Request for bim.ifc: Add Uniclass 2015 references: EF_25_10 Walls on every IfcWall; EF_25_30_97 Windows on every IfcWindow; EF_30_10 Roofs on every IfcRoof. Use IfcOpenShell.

First a look at what the model holds.

```python
import ifcopenshell

model = ifcopenshell.open("bim.ifc")
print(model.schema)
print("classifications:", [c.Name for c in model.by_type("IfcClassification")])
for ifc_class in ("IfcDoor", "IfcRoof", "IfcStair", "IfcWall", "IfcWindow"):
    print(ifc_class, len(model.by_type(ifc_class)))
```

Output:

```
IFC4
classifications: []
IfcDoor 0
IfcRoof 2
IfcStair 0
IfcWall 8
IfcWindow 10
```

```python
import ifcopenshell
import ifcopenshell.api.classification

model = ifcopenshell.open("bim.ifc")

system = ifcopenshell.api.classification.add_classification(model, classification="Uniclass 2015")

codes = {
    "IfcWall": ("EF_25_10", "Walls"),
    "IfcWindow": ("EF_25_30_97", "Windows"),
    "IfcRoof": ("EF_30_10", "Roofs"),
}
for ifc_class, (code, name) in codes.items():
    products = model.by_type(ifc_class)
    ifcopenshell.api.classification.add_reference(
        model, products=products, classification=system, identification=code, name=name
    )
    print(code, len(products))

model.write("bim_updated.ifc")
```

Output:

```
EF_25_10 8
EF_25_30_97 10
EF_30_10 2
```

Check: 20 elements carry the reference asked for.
